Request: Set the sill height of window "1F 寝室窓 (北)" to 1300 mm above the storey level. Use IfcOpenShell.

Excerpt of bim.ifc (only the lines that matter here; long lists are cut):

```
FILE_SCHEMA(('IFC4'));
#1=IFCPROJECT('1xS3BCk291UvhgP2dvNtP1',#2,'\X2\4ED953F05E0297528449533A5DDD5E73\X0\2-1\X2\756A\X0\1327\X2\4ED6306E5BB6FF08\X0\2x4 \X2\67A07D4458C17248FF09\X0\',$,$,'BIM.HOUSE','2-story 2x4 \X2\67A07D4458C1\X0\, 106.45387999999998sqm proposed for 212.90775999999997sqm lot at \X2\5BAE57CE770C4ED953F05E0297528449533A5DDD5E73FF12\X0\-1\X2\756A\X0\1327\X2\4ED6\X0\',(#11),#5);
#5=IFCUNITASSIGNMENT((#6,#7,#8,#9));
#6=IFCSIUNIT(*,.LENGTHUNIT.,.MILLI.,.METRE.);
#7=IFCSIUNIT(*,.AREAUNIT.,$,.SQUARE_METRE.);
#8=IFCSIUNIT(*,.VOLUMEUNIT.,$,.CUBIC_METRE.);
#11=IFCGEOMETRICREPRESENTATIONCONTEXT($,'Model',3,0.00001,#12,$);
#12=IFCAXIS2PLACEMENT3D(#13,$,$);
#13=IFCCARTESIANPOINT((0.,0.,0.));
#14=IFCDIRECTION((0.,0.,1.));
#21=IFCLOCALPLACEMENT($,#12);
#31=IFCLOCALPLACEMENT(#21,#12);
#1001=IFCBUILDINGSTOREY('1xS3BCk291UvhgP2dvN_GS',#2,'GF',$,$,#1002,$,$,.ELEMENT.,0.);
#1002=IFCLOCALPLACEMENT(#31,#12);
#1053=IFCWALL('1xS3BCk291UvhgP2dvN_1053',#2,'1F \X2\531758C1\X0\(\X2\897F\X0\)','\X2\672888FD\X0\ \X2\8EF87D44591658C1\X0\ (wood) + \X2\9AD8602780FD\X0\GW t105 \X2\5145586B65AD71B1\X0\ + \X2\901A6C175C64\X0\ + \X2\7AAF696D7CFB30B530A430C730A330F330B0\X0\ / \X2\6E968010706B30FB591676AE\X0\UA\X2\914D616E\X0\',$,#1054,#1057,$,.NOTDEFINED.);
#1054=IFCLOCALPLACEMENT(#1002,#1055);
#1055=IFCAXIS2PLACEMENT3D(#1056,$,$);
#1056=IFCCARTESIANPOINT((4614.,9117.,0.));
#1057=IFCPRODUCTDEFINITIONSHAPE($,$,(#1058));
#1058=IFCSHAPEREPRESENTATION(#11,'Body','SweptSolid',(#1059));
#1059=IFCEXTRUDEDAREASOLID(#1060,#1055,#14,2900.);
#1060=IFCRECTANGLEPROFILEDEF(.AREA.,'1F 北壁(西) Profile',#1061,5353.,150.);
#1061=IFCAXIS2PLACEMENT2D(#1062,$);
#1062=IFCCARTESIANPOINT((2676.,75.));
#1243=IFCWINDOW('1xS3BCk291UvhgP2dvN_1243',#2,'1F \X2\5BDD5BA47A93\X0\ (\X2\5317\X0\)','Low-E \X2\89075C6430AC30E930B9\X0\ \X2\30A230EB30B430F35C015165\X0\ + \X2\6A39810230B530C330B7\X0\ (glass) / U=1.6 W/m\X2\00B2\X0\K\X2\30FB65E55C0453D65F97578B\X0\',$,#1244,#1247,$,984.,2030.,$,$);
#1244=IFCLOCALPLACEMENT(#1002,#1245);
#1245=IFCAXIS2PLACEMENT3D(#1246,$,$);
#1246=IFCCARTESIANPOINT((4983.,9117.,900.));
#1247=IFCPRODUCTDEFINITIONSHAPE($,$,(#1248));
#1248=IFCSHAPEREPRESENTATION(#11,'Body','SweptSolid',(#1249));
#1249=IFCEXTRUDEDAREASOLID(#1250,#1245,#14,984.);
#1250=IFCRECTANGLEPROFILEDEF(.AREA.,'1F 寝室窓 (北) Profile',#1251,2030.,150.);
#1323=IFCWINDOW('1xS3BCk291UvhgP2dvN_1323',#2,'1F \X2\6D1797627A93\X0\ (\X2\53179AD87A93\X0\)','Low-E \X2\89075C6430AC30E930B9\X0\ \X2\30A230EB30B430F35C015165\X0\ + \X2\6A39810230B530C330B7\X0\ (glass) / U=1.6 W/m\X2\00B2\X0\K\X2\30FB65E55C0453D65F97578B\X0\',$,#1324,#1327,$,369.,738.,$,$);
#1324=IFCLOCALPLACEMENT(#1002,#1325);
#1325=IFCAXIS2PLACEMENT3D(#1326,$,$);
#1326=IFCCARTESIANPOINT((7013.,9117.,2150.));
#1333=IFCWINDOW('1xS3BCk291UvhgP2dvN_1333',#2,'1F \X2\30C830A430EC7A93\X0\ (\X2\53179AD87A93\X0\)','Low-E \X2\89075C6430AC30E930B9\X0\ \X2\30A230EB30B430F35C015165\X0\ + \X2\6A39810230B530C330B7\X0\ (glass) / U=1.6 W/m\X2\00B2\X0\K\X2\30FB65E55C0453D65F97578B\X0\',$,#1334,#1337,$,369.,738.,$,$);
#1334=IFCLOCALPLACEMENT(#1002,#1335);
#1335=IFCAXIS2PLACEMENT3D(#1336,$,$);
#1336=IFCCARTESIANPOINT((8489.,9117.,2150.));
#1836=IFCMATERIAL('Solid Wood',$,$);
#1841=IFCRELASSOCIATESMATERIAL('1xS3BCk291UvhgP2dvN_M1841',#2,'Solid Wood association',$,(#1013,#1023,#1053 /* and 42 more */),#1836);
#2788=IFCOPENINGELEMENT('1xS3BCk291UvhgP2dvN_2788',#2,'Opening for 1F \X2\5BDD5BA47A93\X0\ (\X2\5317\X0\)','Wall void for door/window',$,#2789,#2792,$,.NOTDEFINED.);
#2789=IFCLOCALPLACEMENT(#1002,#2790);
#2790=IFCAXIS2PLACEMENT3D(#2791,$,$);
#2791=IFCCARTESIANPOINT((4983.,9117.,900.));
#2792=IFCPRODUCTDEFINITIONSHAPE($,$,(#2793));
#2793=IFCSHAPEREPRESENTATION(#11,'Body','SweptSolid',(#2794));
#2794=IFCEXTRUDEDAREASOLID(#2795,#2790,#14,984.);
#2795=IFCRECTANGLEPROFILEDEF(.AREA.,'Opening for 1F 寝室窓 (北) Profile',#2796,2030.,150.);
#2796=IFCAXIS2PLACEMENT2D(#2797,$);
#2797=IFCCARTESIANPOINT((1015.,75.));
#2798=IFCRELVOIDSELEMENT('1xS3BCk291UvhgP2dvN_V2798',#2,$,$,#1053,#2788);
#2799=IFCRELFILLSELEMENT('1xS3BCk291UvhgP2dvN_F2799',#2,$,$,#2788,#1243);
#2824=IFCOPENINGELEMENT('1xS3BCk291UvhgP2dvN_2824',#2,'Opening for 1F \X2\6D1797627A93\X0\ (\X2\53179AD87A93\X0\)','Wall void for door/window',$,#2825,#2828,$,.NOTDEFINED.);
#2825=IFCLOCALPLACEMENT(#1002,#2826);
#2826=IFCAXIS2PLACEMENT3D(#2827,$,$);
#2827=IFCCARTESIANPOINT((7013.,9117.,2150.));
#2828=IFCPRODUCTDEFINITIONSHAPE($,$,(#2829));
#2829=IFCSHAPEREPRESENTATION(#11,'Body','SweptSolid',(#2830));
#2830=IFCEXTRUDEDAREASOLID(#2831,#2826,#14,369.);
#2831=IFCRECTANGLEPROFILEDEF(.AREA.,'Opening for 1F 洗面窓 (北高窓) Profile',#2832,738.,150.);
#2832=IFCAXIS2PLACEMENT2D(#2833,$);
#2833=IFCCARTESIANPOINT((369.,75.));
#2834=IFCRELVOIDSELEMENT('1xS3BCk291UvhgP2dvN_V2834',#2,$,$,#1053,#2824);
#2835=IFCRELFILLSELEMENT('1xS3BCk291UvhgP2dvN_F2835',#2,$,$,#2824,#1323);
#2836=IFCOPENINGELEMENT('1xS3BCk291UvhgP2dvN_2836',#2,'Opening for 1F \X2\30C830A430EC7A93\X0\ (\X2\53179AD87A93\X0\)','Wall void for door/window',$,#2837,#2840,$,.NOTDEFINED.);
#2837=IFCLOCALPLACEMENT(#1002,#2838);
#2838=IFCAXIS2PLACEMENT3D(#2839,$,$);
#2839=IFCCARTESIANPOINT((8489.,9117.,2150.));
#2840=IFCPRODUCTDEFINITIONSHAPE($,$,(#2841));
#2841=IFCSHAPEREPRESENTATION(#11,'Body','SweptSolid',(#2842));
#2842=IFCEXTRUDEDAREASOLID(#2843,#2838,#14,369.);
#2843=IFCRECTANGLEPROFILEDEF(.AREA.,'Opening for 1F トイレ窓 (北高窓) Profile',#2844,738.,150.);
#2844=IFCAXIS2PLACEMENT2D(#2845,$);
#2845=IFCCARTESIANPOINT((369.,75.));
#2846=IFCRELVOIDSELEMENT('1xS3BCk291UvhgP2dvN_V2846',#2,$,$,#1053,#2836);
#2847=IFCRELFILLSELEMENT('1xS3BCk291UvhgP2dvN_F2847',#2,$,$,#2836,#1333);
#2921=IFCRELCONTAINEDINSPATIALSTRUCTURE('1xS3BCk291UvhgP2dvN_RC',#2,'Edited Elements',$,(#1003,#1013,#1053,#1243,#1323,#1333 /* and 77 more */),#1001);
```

```python
import numpy as np
import ifcopenshell
import ifcopenshell.api.geometry
import ifcopenshell.geom
import ifcopenshell.util.element
import ifcopenshell.util.placement
import ifcopenshell.util.shape
import ifcopenshell.util.unit

model = ifcopenshell.open("bim.ifc")
unit_scale = ifcopenshell.util.unit.calculate_unit_scale(model)

window = model.by_guid("1xS3BCk291UvhgP2dvN_1243")
opening = window.FillsVoids[0].RelatingOpeningElement
storey = ifcopenshell.util.element.get_container(window, ifc_class="IfcBuildingStorey")
level = ifcopenshell.util.placement.get_local_placement(storey.ObjectPlacement)[2, 3]

# The opening's origin need not be at the sill, so measure its lowest point.
shape = ifcopenshell.geom.create_shape(ifcopenshell.geom.settings(), opening)
bottom = ifcopenshell.util.shape.get_shape_bottom_elevation(shape, shape.geometry) / unit_scale
dz = level + 1.3 / unit_scale - bottom

shift = np.array([0.0, 0.0, dz])
# The window is not placed relative to its opening, so move both.
for product in (opening, window):
    matrix = ifcopenshell.util.placement.get_local_placement(product.ObjectPlacement)
    matrix[:3, 3] += shift
    ifcopenshell.api.geometry.edit_object_placement(model, product=product, matrix=matrix, is_si=False)

print(f"moved by {dz * unit_scale:+.3f} m")

model.write("bim_rev.ifc")
```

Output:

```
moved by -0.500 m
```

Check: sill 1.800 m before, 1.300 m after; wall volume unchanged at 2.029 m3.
